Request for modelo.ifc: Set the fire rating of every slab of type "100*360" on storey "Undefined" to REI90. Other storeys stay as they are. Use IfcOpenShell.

First a look at what the model holds.

```python
import ifcopenshell
import ifcopenshell.util.element

model = ifcopenshell.open("modelo.ifc")
print(model.schema)
storey = next(s for s in model.by_type("IfcBuildingStorey") if s.Name == "Undefined")
slabs = [e for e in ifcopenshell.util.element.get_decomposition(storey) if e.is_a("IfcSlab")]
seen = {}
for e in slabs:
    element_type = ifcopenshell.util.element.get_type(e)
    key = (element_type.Name if element_type != e and element_type else None, ifcopenshell.util.element.get_pset(e, "Pset_SlabCommon", "FireRating"))
    seen[key] = seen.get(key, 0) + 1
for (name, value), count in sorted(seen.items(), key=str):
    print(count, "x", name, "|", value)
```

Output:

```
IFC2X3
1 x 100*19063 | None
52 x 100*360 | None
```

```python
import ifcopenshell
import ifcopenshell.api.pset
import ifcopenshell.util.element

model = ifcopenshell.open("modelo.ifc")

storey = next(s for s in model.by_type("IfcBuildingStorey") if s.Name == "Undefined")
slabs = [e for e in ifcopenshell.util.element.get_decomposition(storey) if e.is_a("IfcSlab")]

count = 0
for e in slabs:
    element_type = ifcopenshell.util.element.get_type(e)
    if element_type in (None, e) or element_type.Name != "100*360":
        continue
    found = ifcopenshell.util.element.get_pset(e, "Pset_SlabCommon", should_inherit=False)
    if found:
        pset = model.by_id(found["id"])
        if len(ifcopenshell.util.element.get_elements_by_pset(pset)) > 1:
            pset = ifcopenshell.api.pset.unshare_pset(model, products=[e], pset=pset)[0]
    else:
        pset = ifcopenshell.api.pset.add_pset(model, product=e, name="Pset_SlabCommon")
    ifcopenshell.api.pset.edit_pset(model, pset=pset, properties={"FireRating": "REI90"})
    count += 1

print(count, "slabs updated")

model.write("modelo_updated.ifc")
```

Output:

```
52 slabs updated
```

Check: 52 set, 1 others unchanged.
